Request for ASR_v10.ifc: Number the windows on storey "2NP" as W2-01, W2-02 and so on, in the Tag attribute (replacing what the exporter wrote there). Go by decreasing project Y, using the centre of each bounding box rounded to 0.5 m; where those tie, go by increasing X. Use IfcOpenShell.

First a look at what the model holds.

```python
import ifcopenshell
import ifcopenshell.util.element
import ifcopenshell.util.placement

model = ifcopenshell.open("ASR_v10.ifc")
print(model.schema)
storey = next(s for s in model.by_type("IfcBuildingStorey") if s.Name == "2NP")
windows = [e for e in ifcopenshell.util.element.get_decomposition(storey) if e.is_a("IfcWindow")]
for e in sorted(windows, key=lambda e: e.id()):
    origin = ifcopenshell.util.placement.get_local_placement(e.ObjectPlacement)[:3, 3]
    print(e.id(), e.Tag, e.Name, origin.round(2) + 0.0, sep=" | ")
```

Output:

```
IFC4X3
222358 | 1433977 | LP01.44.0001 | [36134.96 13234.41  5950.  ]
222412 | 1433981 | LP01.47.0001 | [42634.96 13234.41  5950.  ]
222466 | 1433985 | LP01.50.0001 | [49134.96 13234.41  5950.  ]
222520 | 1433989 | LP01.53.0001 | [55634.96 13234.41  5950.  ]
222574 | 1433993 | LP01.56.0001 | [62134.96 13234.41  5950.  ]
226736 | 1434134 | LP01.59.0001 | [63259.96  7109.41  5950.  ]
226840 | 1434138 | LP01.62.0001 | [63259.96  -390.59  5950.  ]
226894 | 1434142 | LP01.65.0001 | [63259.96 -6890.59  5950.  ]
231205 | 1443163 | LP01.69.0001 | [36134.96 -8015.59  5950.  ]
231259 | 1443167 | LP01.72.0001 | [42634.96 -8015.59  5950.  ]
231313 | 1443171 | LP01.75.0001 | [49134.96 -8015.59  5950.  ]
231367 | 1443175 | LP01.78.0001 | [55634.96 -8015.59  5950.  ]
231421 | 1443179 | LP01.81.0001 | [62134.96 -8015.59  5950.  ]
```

```python
import ifcopenshell
import ifcopenshell.geom
import ifcopenshell.util.element
import ifcopenshell.util.shape

model = ifcopenshell.open("ASR_v10.ifc")
settings = ifcopenshell.geom.settings()
settings.set("use-world-coords", True)


def centre(element):
    shape = ifcopenshell.geom.create_shape(settings, element)
    return ifcopenshell.util.shape.get_bbox_centroid(shape.geometry)


storey = next(s for s in model.by_type("IfcBuildingStorey") if s.Name == "2NP")
windows = [e for e in ifcopenshell.util.element.get_decomposition(storey) if e.is_a("IfcWindow")]

# Insertion points can sit at a corner or the storey origin, so sort by the geometry (in metres).
centres = {e: centre(e) for e in windows}
windows.sort(key=lambda e: (-round(centres[e][1] / 0.5), centres[e][0]))

for i, e in enumerate(windows, start=1):
    number = f"W2-{i:02d}"
    e.Tag = number
    print(e.id(), number)

model.write("ASR_v10_v2.ifc")
```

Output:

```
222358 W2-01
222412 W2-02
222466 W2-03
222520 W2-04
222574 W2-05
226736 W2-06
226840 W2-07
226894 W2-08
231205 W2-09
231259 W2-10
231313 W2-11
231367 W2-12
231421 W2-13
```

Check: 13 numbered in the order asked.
